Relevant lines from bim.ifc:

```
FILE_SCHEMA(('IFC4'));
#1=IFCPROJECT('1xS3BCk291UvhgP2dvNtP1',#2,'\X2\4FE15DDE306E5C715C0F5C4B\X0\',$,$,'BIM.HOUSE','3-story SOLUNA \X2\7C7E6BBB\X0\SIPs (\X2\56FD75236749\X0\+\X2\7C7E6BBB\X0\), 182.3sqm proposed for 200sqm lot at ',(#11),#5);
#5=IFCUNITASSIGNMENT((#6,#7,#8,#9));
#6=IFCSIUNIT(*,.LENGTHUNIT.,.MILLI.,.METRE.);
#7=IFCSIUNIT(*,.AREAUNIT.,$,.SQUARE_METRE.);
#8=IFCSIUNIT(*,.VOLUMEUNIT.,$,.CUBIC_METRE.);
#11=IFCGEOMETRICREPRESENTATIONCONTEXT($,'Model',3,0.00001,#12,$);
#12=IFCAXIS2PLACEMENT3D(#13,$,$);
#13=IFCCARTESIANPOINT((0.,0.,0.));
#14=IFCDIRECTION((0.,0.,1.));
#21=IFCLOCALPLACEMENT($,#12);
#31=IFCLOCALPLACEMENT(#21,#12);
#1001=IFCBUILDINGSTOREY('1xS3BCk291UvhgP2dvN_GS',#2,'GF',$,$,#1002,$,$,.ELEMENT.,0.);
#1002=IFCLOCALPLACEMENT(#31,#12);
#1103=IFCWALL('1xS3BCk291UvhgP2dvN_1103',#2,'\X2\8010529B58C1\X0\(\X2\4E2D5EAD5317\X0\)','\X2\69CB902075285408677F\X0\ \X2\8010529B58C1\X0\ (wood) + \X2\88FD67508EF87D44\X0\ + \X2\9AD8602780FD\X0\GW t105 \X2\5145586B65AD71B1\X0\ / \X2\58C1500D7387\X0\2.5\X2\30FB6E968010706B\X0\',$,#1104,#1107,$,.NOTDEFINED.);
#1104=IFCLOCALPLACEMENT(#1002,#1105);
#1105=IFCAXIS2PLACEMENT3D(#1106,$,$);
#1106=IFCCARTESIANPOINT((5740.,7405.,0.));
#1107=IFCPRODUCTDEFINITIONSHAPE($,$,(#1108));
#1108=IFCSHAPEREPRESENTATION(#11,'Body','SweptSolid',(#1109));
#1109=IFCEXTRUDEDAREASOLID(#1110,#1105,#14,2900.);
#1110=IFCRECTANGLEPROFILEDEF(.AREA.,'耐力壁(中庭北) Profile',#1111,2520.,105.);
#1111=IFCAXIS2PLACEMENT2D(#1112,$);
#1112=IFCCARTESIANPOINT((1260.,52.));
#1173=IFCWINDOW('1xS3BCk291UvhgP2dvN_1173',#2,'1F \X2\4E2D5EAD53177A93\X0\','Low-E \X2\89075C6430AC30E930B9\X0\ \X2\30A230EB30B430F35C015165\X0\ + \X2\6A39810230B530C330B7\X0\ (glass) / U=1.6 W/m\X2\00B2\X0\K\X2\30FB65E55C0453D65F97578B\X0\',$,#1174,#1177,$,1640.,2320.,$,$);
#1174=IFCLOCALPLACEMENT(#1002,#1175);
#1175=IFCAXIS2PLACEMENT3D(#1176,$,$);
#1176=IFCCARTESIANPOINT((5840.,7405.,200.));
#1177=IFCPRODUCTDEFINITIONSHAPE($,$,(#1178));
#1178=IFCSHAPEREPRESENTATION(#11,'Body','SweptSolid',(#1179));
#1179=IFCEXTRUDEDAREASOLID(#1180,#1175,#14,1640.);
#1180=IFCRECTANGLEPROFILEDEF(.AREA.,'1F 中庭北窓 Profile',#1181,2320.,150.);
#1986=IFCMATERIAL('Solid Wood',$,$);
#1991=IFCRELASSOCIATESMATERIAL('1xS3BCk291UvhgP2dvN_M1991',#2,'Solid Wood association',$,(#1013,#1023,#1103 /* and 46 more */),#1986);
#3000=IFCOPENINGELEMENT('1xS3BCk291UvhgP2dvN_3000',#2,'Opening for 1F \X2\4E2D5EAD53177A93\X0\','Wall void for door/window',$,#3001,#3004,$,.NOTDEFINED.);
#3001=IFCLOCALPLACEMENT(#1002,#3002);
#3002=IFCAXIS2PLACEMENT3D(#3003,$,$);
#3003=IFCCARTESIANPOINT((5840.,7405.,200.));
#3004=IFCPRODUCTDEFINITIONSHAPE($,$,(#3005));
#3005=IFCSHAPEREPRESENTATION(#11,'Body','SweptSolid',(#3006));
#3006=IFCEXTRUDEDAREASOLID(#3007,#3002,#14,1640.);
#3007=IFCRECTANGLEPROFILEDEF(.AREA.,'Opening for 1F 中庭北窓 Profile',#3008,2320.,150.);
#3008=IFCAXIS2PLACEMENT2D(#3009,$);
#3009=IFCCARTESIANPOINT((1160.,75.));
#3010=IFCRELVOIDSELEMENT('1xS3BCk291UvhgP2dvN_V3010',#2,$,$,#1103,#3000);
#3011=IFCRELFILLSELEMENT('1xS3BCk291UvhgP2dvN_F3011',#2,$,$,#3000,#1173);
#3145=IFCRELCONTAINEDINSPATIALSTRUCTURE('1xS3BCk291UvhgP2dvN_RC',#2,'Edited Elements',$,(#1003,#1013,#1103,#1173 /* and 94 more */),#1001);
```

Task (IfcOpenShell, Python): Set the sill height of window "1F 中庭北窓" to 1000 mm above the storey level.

```python
import numpy as np
import ifcopenshell
import ifcopenshell.api.geometry
import ifcopenshell.geom
import ifcopenshell.util.element
import ifcopenshell.util.placement
import ifcopenshell.util.shape
import ifcopenshell.util.unit

model = ifcopenshell.open("bim.ifc")
unit_scale = ifcopenshell.util.unit.calculate_unit_scale(model)

window = model.by_guid("1xS3BCk291UvhgP2dvN_1173")
opening = window.FillsVoids[0].RelatingOpeningElement
storey = ifcopenshell.util.element.get_container(window, ifc_class="IfcBuildingStorey")
level = ifcopenshell.util.placement.get_local_placement(storey.ObjectPlacement)[2, 3]

# The opening's origin need not be at the sill, so measure its lowest point.
shape = ifcopenshell.geom.create_shape(ifcopenshell.geom.settings(), opening)
bottom = ifcopenshell.util.shape.get_shape_bottom_elevation(shape, shape.geometry) / unit_scale
dz = level + 1 / unit_scale - bottom

shift = np.array([0.0, 0.0, dz])
# The window is not placed relative to its opening, so move both.
for product in (opening, window):
    matrix = ifcopenshell.util.placement.get_local_placement(product.ObjectPlacement)
    matrix[:3, 3] += shift
    ifcopenshell.api.geometry.edit_object_placement(model, product=product, matrix=matrix, is_si=False)

print(f"moved by {dz * unit_scale:+.3f} m")

model.write("bim-out.ifc")
```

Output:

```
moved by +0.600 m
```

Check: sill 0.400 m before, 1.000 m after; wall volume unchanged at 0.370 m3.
